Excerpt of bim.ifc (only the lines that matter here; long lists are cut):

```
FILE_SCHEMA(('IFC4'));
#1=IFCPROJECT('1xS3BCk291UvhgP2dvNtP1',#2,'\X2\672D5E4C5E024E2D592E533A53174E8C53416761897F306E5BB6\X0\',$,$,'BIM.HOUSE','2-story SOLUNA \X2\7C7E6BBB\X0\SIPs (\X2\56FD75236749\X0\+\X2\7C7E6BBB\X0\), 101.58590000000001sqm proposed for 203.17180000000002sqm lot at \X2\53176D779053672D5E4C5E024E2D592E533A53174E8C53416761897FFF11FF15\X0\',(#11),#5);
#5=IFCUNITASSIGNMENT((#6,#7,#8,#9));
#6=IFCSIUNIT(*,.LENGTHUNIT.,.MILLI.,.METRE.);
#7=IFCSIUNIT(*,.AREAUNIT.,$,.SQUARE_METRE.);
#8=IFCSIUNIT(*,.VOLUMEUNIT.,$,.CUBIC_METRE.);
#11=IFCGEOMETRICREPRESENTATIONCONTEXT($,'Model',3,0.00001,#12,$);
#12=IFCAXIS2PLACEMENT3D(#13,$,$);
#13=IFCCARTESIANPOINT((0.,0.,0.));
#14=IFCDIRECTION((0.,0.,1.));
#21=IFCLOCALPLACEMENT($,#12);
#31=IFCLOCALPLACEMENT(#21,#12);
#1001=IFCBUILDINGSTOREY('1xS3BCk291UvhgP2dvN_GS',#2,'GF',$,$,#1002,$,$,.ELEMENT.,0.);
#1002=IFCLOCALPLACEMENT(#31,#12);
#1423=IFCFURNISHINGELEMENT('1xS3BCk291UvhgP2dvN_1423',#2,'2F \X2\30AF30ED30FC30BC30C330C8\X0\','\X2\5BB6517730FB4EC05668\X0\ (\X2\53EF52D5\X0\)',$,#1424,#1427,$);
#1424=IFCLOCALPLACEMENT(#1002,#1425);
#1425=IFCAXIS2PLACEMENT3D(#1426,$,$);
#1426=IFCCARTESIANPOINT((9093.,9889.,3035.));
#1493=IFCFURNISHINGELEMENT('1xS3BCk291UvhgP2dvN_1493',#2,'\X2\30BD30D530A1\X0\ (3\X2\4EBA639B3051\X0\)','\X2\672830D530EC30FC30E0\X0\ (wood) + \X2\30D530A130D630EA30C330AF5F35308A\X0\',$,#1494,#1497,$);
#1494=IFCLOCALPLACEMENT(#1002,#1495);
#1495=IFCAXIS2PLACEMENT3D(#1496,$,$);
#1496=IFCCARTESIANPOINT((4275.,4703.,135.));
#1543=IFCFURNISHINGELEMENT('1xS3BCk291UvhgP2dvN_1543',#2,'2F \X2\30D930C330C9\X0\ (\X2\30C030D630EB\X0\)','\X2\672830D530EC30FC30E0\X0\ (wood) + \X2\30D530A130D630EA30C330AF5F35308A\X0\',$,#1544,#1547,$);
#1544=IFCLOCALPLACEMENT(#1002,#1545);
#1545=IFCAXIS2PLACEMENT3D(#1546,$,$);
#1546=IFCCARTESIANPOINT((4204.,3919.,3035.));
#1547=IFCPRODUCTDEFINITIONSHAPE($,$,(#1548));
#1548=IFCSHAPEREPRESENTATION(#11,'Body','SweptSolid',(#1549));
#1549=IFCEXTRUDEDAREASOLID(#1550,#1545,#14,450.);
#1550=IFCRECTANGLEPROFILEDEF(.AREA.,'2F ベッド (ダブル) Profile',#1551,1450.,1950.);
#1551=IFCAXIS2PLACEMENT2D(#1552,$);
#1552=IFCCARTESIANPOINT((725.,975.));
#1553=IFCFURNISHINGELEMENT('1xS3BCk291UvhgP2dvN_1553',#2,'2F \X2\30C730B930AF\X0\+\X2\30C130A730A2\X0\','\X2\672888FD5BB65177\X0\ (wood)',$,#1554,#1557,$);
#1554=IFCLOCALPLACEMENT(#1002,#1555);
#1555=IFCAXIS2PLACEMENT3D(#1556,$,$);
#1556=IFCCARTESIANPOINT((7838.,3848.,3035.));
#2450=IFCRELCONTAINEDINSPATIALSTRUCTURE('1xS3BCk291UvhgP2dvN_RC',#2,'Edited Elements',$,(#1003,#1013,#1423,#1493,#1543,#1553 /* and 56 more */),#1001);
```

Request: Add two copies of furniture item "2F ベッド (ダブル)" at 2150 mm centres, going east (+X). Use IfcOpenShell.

```python
import numpy as np
import ifcopenshell
import ifcopenshell.api.geometry
import ifcopenshell.api.root
import ifcopenshell.util.element
import ifcopenshell.util.placement
import ifcopenshell.util.unit

model = ifcopenshell.open("bim.ifc")
unit_scale = ifcopenshell.util.unit.calculate_unit_scale(model)


def reuse_history(source, copy):
    """copy_class also copies each property set's owner history, people and application; keep the originals."""
    for rel in copy.IsDefinedBy:
        if rel.is_a("IfcRelDefinesByProperties") and (history := rel.RelatingPropertyDefinition.OwnerHistory):
            rel.RelatingPropertyDefinition.OwnerHistory = source.OwnerHistory
            ifcopenshell.util.element.remove_deep2(model, history)


source = model.by_guid("1xS3BCk291UvhgP2dvN_1543")
base = ifcopenshell.util.placement.get_local_placement(source.ObjectPlacement)
step = np.array([1.0, 0.0, 0.0]) * 2.15 / unit_scale

for i in range(1, 3):
    copy = ifcopenshell.api.root.copy_class(model, product=source)
    copy.Representation = ifcopenshell.util.element.copy_deep(
        model, source.Representation, exclude=["IfcGeometricRepresentationContext", "IfcRepresentationMap"]
    )
    reuse_history(source, copy)
    matrix = base.copy()
    matrix[:3, 3] += i * step
    print("added at", matrix[:3, 3].round(3) + 0.0)
    ifcopenshell.api.geometry.edit_object_placement(model, product=copy, matrix=matrix, is_si=False)

model.write("bim_updated.ifc")
```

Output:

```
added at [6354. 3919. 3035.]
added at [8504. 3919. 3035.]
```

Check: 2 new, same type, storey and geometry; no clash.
